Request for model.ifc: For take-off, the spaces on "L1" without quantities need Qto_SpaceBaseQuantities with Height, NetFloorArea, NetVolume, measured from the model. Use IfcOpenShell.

First a look at what the model holds.

```python
import ifcopenshell
import ifcopenshell.util.element
import ifcopenshell.util.unit

model = ifcopenshell.open("model.ifc")
print(model.schema)
for unit_type in ("LENGTHUNIT", "AREAUNIT", "VOLUMEUNIT"):
    print(unit_type, ifcopenshell.util.unit.calculate_unit_scale(model, unit_type))
storey = next(s for s in model.by_type("IfcBuildingStorey") if s.Name == "L1")
spaces = [e for e in ifcopenshell.util.element.get_decomposition(storey) if e.is_a("IfcSpace")]
for e in sorted(spaces, key=lambda e: e.id()):
    print(e.id(), e.is_a(), e.Name, list(ifcopenshell.util.element.get_psets(e, qtos_only=True)), sep=" | ")
```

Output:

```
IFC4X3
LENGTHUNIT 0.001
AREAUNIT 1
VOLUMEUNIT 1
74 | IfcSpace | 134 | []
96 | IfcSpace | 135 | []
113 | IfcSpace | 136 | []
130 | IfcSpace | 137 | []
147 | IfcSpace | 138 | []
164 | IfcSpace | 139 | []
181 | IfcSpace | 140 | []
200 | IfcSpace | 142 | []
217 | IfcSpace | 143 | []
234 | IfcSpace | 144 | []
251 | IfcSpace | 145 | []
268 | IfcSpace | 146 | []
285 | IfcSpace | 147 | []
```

```python
import ifcopenshell
import ifcopenshell.api.pset
import ifcopenshell.geom
import ifcopenshell.util.element
import ifcopenshell.util.shape
import ifcopenshell.util.unit

model = ifcopenshell.open("model.ifc")
unit_scale = ifcopenshell.util.unit.calculate_unit_scale(model)
area_scale = ifcopenshell.util.unit.calculate_unit_scale(model, "AREAUNIT")
volume_scale = ifcopenshell.util.unit.calculate_unit_scale(model, "VOLUMEUNIT")
settings = ifcopenshell.geom.settings()

storey = next(s for s in model.by_type("IfcBuildingStorey") if s.Name == "L1")
spaces = [e for e in ifcopenshell.util.element.get_decomposition(storey) if e.is_a("IfcSpace")]

for e in sorted(spaces, key=lambda e: e.id()):
    if ifcopenshell.util.element.get_psets(e, qtos_only=True, should_inherit=False):
        continue
    # Geometry comes back in metres, in the element's own axes.
    shape = ifcopenshell.geom.create_shape(settings, e)
    values = {
        "Height": ifcopenshell.util.shape.get_z(shape.geometry) / unit_scale,
        "NetFloorArea": ifcopenshell.util.shape.get_footprint_area(shape.geometry) / area_scale,
        "NetVolume": ifcopenshell.util.shape.get_volume(shape.geometry) / volume_scale,
    }
    qto = ifcopenshell.api.pset.add_qto(model, product=e, name="Qto_SpaceBaseQuantities")
    ifcopenshell.api.pset.edit_qto(model, qto=qto, properties=values)
    print(e.id(), {k: round(v, 3) for k, v in values.items()})

model.write("model-out.ifc")
```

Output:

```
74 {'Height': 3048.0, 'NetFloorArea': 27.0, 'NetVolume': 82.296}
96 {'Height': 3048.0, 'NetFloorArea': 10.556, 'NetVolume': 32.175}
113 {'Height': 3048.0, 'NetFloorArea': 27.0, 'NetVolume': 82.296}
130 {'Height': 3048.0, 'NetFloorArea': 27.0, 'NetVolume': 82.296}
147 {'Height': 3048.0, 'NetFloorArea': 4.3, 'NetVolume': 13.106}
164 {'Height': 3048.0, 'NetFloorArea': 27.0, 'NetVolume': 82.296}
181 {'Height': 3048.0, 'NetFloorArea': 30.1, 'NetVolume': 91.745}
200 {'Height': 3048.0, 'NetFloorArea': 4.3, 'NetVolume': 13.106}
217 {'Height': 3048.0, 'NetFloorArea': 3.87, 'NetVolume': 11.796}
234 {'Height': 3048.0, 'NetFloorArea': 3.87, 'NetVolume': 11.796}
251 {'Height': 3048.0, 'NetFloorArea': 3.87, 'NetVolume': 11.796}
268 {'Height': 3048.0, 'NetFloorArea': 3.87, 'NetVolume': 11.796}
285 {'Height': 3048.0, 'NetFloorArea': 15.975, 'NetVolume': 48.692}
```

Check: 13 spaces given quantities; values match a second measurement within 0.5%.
